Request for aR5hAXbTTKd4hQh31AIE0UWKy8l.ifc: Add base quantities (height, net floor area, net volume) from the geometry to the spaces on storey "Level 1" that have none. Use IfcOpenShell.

First a look at what the model holds.

```python
import ifcopenshell
import ifcopenshell.util.element
import ifcopenshell.util.unit

model = ifcopenshell.open("aR5hAXbTTKd4hQh31AIE0UWKy8l.ifc")
print(model.schema)
for unit_type in ("LENGTHUNIT", "AREAUNIT", "VOLUMEUNIT"):
    print(unit_type, ifcopenshell.util.unit.calculate_unit_scale(model, unit_type))
storey = next(s for s in model.by_type("IfcBuildingStorey") if s.Name == "Level 1")
spaces = [e for e in ifcopenshell.util.element.get_decomposition(storey) if e.is_a("IfcSpace")]
for e in sorted(spaces, key=lambda e: e.id()):
    print(e.id(), e.is_a(), e.Name, list(ifcopenshell.util.element.get_psets(e, qtos_only=True)), sep=" | ")
```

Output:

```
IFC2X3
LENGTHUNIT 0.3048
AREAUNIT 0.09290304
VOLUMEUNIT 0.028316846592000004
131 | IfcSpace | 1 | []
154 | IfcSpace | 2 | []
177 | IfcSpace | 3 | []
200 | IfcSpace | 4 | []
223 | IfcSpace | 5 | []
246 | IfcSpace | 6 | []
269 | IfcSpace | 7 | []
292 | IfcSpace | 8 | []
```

```python
import ifcopenshell
import ifcopenshell.api.pset
import ifcopenshell.geom
import ifcopenshell.util.element
import ifcopenshell.util.shape
import ifcopenshell.util.unit

model = ifcopenshell.open("aR5hAXbTTKd4hQh31AIE0UWKy8l.ifc")
unit_scale = ifcopenshell.util.unit.calculate_unit_scale(model)
area_scale = ifcopenshell.util.unit.calculate_unit_scale(model, "AREAUNIT")
volume_scale = ifcopenshell.util.unit.calculate_unit_scale(model, "VOLUMEUNIT")
settings = ifcopenshell.geom.settings()

storey = next(s for s in model.by_type("IfcBuildingStorey") if s.Name == "Level 1")
spaces = [e for e in ifcopenshell.util.element.get_decomposition(storey) if e.is_a("IfcSpace")]

for e in sorted(spaces, key=lambda e: e.id()):
    if ifcopenshell.util.element.get_psets(e, qtos_only=True, should_inherit=False):
        continue
    # Geometry comes back in metres, in the element's own axes.
    shape = ifcopenshell.geom.create_shape(settings, e)
    values = {
        "Height": ifcopenshell.util.shape.get_z(shape.geometry) / unit_scale,
        "NetFloorArea": ifcopenshell.util.shape.get_footprint_area(shape.geometry) / area_scale,
        "NetVolume": ifcopenshell.util.shape.get_volume(shape.geometry) / volume_scale,
    }
    qto = ifcopenshell.api.pset.add_qto(model, product=e, name="BaseQuantities")
    ifcopenshell.api.pset.edit_qto(model, qto=qto, properties=values)
    print(e.id(), {k: round(v, 3) for k, v in values.items()})

model.write("aR5hAXbTTKd4hQh31AIE0UWKy8l_rev.ifc")
```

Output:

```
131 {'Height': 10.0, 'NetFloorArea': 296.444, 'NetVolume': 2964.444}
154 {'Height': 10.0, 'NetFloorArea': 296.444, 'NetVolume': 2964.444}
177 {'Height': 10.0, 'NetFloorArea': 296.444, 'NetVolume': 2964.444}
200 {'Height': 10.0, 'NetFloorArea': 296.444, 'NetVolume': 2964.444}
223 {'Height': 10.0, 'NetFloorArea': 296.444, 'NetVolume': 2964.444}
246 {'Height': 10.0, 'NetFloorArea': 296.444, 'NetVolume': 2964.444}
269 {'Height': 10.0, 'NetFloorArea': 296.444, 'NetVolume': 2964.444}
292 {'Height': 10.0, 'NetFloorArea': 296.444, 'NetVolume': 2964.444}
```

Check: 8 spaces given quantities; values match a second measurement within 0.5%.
